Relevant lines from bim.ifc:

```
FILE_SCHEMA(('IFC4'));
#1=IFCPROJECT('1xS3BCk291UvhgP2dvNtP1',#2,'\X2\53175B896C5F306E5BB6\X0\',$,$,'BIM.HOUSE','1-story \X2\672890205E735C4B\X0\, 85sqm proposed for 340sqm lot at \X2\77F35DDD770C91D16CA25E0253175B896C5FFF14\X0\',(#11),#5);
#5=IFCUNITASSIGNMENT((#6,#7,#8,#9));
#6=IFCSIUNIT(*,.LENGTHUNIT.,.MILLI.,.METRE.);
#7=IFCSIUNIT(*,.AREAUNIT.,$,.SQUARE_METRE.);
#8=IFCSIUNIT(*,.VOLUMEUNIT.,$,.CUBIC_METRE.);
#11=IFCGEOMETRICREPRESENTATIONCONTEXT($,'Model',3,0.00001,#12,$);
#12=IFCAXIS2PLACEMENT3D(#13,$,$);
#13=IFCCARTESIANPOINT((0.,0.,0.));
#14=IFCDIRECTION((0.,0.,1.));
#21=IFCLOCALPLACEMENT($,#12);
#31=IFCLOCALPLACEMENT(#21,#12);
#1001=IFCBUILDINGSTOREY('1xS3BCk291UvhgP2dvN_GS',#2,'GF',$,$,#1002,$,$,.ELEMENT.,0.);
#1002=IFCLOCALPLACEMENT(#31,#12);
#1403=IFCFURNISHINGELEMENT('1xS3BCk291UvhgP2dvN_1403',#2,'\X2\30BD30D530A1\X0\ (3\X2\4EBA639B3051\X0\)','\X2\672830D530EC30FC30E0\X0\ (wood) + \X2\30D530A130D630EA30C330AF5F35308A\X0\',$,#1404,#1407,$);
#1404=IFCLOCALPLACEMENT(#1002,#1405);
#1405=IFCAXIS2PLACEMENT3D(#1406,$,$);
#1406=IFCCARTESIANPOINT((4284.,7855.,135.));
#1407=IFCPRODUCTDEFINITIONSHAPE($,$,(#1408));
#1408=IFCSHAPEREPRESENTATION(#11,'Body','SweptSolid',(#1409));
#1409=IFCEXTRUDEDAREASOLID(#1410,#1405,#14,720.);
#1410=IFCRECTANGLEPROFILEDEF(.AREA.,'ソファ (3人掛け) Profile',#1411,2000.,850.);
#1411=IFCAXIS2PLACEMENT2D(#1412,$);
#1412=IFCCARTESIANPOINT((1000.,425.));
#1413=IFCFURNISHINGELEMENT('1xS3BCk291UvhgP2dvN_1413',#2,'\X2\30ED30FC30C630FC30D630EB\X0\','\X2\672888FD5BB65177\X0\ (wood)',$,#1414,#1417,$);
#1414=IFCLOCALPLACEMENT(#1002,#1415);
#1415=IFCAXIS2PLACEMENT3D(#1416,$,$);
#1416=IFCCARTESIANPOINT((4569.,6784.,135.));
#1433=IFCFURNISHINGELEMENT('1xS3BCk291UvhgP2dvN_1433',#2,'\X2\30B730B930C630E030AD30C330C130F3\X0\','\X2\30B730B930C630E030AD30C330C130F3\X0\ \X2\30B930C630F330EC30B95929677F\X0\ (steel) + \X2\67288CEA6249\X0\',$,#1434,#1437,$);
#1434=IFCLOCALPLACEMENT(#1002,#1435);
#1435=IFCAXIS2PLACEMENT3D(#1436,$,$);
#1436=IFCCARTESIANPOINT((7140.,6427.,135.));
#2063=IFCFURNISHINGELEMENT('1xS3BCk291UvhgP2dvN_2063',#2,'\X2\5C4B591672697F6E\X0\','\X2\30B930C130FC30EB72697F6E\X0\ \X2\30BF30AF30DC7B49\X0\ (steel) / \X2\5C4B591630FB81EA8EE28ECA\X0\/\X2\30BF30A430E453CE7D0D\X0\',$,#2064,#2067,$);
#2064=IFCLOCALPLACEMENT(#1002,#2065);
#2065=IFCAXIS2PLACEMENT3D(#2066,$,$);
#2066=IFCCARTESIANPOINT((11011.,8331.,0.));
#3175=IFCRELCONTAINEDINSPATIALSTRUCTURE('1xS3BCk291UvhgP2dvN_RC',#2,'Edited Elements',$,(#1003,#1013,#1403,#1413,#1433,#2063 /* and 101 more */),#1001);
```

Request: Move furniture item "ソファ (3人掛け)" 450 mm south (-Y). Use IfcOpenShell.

```python
import ifcopenshell
import ifcopenshell.api.geometry
import ifcopenshell.util.placement

model = ifcopenshell.open("bim.ifc")

item = model.by_guid("1xS3BCk291UvhgP2dvN_1403")
matrix = ifcopenshell.util.placement.get_local_placement(item.ObjectPlacement)
matrix[1, 3] -= 450.0
ifcopenshell.api.geometry.edit_object_placement(model, product=item, matrix=matrix, is_si=False)

print(ifcopenshell.util.placement.get_local_placement(item.ObjectPlacement).round(3) + 0.0)

model.write("bim_updated.ifc")
```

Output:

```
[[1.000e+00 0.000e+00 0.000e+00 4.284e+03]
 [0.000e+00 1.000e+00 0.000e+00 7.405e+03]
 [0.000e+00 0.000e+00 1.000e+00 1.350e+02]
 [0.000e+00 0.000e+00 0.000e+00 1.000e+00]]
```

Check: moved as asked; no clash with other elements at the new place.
